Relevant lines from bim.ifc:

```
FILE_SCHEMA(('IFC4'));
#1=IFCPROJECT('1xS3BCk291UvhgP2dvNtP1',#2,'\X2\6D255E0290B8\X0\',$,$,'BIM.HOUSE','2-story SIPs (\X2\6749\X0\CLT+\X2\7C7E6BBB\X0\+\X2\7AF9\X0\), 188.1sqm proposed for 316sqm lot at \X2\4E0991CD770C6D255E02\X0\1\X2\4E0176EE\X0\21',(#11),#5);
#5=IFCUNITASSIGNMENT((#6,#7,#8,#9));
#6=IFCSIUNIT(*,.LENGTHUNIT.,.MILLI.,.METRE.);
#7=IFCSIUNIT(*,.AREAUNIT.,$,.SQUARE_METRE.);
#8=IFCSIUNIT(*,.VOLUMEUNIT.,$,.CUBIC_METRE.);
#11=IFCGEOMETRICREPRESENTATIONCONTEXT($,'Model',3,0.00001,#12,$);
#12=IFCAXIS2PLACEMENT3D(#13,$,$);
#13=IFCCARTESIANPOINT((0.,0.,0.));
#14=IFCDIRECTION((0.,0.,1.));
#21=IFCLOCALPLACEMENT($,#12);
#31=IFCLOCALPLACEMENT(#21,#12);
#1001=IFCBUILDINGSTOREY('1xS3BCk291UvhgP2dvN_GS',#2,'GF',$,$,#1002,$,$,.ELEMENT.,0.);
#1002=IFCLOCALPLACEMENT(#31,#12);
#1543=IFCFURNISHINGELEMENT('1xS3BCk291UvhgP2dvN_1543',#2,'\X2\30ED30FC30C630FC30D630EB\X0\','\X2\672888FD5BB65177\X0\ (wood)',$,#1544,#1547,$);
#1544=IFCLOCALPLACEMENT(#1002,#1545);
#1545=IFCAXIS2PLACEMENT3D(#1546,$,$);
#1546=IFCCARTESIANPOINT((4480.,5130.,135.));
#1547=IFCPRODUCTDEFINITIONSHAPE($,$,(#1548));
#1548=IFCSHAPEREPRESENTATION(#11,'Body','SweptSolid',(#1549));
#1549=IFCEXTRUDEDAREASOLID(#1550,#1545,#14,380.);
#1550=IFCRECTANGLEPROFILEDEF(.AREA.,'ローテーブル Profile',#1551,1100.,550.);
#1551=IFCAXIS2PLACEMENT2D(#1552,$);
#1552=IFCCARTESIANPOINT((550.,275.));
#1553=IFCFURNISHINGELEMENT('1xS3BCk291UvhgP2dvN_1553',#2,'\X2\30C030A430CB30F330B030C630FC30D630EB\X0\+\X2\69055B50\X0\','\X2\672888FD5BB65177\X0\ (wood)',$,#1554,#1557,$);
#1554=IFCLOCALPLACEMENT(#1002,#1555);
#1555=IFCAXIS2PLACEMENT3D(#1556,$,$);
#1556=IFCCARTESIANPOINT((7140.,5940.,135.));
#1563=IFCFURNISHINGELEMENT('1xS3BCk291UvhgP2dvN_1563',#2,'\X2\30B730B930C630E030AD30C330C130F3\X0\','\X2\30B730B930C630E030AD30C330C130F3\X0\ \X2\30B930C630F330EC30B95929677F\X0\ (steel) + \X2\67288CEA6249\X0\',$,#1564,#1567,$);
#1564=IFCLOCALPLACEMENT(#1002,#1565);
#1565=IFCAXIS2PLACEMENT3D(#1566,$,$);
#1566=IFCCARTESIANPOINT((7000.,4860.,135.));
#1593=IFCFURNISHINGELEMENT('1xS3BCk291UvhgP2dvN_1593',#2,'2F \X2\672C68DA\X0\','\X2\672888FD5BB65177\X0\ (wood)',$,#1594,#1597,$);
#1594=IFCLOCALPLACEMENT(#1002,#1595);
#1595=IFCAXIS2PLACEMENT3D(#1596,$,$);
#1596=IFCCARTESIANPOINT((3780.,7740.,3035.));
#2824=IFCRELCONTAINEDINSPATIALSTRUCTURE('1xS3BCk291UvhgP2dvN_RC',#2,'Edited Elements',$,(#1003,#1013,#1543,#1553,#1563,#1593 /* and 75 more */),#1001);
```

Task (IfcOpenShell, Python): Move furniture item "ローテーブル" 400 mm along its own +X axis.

```python
import ifcopenshell
import ifcopenshell.api.geometry
import ifcopenshell.util.placement
import ifcopenshell.util.unit

model = ifcopenshell.open("bim.ifc")
unit_scale = ifcopenshell.util.unit.calculate_unit_scale(model)

item = model.by_guid("1xS3BCk291UvhgP2dvN_1543")
matrix = ifcopenshell.util.placement.get_local_placement(item.ObjectPlacement)
matrix[:3, 3] += matrix[:3, 0] * 0.4 / unit_scale
ifcopenshell.api.geometry.edit_object_placement(model, product=item, matrix=matrix, is_si=False)

print(ifcopenshell.util.placement.get_local_placement(item.ObjectPlacement).round(3) + 0.0)

model.write("bim-out.ifc")
```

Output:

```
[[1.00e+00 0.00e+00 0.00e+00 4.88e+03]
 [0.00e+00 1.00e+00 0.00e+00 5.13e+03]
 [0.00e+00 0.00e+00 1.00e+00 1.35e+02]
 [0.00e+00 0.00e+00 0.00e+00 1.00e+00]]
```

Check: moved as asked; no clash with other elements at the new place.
